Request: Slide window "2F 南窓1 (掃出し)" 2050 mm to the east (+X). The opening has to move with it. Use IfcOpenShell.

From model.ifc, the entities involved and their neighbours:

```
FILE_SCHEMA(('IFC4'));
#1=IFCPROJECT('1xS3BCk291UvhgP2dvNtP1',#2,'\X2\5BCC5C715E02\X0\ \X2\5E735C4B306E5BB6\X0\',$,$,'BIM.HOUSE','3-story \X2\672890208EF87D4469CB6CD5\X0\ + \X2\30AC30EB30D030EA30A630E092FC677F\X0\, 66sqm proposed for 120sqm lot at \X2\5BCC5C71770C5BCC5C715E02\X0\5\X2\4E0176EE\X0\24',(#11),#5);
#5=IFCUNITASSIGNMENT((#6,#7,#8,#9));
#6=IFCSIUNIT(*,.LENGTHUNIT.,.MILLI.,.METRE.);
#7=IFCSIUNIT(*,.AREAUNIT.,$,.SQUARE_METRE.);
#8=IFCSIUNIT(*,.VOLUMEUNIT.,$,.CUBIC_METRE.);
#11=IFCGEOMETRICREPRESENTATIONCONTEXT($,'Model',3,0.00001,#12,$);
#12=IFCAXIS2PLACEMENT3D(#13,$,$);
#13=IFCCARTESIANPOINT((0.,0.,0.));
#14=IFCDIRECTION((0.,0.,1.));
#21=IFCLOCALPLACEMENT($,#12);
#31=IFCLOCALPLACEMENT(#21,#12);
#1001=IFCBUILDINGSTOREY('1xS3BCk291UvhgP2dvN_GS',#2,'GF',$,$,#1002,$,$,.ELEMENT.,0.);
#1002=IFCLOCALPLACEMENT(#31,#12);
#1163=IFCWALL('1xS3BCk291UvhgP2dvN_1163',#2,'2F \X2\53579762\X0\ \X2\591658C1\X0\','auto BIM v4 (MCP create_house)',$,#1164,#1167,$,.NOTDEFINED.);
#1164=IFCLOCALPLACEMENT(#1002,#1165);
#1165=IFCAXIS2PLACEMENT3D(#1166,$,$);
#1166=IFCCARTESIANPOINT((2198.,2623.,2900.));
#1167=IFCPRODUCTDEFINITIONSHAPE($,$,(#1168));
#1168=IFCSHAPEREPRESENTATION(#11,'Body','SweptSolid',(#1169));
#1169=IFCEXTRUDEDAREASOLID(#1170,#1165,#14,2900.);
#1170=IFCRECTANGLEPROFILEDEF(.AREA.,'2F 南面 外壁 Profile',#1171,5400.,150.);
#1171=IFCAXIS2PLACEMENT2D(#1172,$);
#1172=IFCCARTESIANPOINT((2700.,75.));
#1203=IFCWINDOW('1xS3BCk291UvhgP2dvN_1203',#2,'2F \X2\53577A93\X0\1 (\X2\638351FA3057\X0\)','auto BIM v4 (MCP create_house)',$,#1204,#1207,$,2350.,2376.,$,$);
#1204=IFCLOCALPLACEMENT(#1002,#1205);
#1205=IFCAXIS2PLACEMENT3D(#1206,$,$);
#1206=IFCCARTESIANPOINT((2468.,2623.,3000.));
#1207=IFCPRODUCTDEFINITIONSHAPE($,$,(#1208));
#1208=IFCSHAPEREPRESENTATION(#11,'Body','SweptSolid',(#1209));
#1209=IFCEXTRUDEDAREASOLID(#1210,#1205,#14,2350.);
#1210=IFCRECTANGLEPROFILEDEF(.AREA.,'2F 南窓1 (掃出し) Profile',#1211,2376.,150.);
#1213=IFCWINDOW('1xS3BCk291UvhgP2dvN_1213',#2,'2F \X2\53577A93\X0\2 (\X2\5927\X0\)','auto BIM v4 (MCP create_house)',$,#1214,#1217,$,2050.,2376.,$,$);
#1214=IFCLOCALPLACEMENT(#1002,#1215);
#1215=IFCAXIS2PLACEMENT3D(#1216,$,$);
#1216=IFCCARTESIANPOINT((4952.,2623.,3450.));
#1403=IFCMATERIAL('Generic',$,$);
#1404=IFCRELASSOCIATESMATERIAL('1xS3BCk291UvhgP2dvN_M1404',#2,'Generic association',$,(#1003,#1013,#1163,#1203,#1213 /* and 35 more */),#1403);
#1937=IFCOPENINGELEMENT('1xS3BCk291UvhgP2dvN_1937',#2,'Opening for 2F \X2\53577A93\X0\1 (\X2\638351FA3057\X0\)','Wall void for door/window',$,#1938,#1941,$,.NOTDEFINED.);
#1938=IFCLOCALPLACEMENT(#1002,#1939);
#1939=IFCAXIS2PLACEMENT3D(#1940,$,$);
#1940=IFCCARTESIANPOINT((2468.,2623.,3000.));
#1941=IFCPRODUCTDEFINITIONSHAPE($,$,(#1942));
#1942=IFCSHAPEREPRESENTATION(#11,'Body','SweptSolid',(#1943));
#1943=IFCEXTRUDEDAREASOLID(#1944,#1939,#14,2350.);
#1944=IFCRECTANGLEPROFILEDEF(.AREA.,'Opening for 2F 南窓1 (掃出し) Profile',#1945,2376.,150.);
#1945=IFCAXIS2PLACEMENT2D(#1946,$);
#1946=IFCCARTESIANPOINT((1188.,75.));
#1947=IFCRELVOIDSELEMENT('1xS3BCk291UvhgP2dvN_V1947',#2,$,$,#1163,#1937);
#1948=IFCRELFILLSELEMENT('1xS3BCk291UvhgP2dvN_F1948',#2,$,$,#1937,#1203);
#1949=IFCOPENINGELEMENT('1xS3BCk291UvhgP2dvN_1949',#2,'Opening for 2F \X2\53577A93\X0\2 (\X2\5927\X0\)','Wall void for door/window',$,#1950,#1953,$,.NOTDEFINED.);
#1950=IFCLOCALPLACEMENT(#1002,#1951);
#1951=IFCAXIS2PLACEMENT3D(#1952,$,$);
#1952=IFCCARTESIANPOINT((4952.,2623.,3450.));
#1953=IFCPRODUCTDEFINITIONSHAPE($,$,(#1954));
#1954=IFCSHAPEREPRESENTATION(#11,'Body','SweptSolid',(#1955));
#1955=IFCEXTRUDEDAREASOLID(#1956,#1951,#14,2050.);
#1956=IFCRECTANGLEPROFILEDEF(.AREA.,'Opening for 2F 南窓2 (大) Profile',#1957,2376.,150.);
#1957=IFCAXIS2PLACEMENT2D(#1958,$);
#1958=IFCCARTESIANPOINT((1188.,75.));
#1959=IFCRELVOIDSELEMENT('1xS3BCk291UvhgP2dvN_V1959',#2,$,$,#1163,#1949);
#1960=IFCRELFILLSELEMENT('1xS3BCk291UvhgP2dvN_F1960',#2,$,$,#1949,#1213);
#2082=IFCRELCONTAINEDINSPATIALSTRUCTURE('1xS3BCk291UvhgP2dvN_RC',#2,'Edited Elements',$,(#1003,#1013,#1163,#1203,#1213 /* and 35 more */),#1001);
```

```python
import ifcopenshell
import ifcopenshell.api.geometry
import ifcopenshell.util.placement

model = ifcopenshell.open("model.ifc")

window = model.by_id(1203)
opening = window.FillsVoids[0].RelatingOpeningElement
wall = opening.VoidsElements[0].RelatingBuildingElement

wall_matrix = ifcopenshell.util.placement.get_local_placement(wall.ObjectPlacement)
shift = wall_matrix[:3, 0] * 2050.0
before = ifcopenshell.util.placement.get_local_placement(window.ObjectPlacement)[:3, 3].copy()

# The window is not placed relative to its opening, so move both.
for product in (opening, window):
    matrix = ifcopenshell.util.placement.get_local_placement(product.ObjectPlacement)
    matrix[:3, 3] += shift
    ifcopenshell.api.geometry.edit_object_placement(model, product=product, matrix=matrix, is_si=False)

after = ifcopenshell.util.placement.get_local_placement(window.ObjectPlacement)[:3, 3]
print("window moved by", (after - before).round(3) + 0.0)

model.write("model_v2.ifc")
```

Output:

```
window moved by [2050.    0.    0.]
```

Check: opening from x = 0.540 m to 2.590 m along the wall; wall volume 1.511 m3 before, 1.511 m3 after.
